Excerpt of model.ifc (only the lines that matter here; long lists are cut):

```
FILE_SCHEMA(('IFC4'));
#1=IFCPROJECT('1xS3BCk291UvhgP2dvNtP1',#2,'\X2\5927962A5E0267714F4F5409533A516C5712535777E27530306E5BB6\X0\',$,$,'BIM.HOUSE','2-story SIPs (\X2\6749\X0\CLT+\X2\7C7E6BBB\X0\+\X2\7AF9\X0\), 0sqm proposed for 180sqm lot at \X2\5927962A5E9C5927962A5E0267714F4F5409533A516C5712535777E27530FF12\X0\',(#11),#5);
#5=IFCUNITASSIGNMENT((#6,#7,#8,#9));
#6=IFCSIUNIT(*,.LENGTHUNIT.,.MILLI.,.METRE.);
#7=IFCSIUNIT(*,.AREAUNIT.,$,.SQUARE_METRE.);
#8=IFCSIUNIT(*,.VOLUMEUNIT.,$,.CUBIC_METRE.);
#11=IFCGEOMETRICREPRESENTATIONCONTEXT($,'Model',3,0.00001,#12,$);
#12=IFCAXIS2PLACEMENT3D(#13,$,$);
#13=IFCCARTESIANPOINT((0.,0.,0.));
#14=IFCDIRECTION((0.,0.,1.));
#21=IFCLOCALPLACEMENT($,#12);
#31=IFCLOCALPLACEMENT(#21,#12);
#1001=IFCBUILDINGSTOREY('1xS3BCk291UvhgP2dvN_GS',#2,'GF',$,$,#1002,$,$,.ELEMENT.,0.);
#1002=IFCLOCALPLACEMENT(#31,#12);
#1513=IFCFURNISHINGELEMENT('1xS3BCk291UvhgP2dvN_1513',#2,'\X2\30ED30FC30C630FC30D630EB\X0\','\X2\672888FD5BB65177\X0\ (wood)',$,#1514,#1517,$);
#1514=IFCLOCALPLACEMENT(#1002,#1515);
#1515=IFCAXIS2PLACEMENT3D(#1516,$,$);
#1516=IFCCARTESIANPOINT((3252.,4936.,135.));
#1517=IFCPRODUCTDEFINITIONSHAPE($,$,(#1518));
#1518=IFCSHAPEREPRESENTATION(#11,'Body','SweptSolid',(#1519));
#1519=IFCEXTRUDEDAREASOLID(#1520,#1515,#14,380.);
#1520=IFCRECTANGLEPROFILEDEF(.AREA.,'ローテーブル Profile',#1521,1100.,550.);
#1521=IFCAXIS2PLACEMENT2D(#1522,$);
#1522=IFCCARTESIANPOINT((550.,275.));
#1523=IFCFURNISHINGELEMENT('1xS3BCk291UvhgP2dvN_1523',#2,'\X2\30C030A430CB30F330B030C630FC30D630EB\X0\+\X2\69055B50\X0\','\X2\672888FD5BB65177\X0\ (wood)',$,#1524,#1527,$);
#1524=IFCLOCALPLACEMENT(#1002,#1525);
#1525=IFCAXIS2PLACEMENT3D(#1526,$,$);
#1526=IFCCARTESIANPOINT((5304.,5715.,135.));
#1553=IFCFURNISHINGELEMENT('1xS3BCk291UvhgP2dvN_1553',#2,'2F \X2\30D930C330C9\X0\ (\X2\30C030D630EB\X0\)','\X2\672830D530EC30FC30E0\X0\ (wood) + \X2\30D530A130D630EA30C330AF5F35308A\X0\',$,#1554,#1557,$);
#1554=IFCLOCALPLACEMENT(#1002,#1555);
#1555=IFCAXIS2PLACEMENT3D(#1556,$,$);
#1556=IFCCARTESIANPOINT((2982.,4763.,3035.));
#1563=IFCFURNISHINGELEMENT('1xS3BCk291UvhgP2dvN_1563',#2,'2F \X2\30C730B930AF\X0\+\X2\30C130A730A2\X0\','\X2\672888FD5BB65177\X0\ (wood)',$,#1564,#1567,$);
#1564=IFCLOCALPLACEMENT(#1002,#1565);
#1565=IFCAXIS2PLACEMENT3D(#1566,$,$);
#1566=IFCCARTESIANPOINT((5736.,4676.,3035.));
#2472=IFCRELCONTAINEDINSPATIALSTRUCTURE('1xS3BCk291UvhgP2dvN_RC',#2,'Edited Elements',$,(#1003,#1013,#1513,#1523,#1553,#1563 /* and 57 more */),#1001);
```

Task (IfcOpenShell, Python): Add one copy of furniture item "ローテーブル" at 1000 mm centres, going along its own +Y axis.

```python
import ifcopenshell
import ifcopenshell.api.geometry
import ifcopenshell.api.root
import ifcopenshell.util.element
import ifcopenshell.util.placement
import ifcopenshell.util.unit

model = ifcopenshell.open("model.ifc")
unit_scale = ifcopenshell.util.unit.calculate_unit_scale(model)


def reuse_history(source, copy):
    """copy_class also copies each property set's owner history, people and application; keep the originals."""
    for rel in copy.IsDefinedBy:
        if rel.is_a("IfcRelDefinesByProperties") and (history := rel.RelatingPropertyDefinition.OwnerHistory):
            rel.RelatingPropertyDefinition.OwnerHistory = source.OwnerHistory
            ifcopenshell.util.element.remove_deep2(model, history)


source = model.by_id(1513)
base = ifcopenshell.util.placement.get_local_placement(source.ObjectPlacement)
step = base[:3, 1] * 1 / unit_scale

for i in range(1, 2):
    copy = ifcopenshell.api.root.copy_class(model, product=source)
    copy.Representation = ifcopenshell.util.element.copy_deep(
        model, source.Representation, exclude=["IfcGeometricRepresentationContext", "IfcRepresentationMap"]
    )
    reuse_history(source, copy)
    matrix = base.copy()
    matrix[:3, 3] += i * step
    print("added at", matrix[:3, 3].round(3) + 0.0)
    ifcopenshell.api.geometry.edit_object_placement(model, product=copy, matrix=matrix, is_si=False)

model.write("model_edited.ifc")
```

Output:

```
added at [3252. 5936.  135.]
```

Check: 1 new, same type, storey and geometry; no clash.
